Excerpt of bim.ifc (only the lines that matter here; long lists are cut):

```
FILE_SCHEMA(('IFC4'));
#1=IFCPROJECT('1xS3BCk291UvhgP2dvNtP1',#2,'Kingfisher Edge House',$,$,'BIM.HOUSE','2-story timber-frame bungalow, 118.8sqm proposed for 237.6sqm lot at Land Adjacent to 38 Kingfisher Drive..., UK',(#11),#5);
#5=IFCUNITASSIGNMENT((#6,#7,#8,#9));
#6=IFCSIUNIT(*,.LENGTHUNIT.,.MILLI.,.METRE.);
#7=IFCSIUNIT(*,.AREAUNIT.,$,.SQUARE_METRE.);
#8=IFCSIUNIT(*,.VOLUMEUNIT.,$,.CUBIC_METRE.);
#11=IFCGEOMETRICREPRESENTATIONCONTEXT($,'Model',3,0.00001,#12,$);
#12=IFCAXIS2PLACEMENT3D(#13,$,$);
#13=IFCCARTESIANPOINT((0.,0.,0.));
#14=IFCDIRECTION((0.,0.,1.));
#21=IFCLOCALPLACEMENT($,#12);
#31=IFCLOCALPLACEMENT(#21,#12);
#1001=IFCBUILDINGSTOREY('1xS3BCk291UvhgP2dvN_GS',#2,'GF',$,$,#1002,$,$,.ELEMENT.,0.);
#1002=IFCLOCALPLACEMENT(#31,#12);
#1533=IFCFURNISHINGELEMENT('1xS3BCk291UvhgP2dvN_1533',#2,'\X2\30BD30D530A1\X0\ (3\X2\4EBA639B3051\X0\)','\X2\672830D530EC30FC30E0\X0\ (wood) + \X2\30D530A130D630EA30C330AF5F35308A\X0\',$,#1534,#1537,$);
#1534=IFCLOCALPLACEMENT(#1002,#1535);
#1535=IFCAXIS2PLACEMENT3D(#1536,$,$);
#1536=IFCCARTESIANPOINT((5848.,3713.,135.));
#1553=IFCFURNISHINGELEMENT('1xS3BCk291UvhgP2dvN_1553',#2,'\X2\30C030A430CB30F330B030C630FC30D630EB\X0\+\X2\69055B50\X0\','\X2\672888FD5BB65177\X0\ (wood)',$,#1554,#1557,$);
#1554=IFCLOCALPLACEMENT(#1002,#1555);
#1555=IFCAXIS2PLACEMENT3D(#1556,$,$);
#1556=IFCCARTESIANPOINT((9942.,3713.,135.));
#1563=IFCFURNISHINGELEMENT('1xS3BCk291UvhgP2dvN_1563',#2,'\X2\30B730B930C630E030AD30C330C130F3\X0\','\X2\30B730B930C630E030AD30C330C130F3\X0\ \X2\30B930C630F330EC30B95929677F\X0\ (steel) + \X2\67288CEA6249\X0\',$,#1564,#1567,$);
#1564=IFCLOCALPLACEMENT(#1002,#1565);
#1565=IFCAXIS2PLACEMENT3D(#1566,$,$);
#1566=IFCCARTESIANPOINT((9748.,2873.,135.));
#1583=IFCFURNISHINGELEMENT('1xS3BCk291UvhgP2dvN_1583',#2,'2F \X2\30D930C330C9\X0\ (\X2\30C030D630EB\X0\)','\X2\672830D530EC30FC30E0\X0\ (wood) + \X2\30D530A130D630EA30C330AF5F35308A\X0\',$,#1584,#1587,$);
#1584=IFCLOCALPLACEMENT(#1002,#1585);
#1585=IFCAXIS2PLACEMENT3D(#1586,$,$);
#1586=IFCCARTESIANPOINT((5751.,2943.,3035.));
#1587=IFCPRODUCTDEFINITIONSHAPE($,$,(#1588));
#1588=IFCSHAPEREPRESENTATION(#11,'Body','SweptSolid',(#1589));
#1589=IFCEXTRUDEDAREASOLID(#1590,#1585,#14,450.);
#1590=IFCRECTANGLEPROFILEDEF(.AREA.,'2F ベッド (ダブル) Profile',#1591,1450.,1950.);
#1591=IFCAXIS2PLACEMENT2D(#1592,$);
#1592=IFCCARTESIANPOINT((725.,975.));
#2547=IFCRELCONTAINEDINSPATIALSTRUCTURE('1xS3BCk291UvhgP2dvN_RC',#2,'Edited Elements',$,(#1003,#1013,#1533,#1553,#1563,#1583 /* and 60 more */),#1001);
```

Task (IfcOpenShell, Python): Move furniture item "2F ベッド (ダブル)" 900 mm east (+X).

```python
import ifcopenshell
import ifcopenshell.api.geometry
import ifcopenshell.util.placement
import ifcopenshell.util.unit

model = ifcopenshell.open("bim.ifc")
unit_scale = ifcopenshell.util.unit.calculate_unit_scale(model)

item = model.by_guid("1xS3BCk291UvhgP2dvN_1583")
matrix = ifcopenshell.util.placement.get_local_placement(item.ObjectPlacement)
matrix[0, 3] += 0.9 / unit_scale
ifcopenshell.api.geometry.edit_object_placement(model, product=item, matrix=matrix, is_si=False)

print(ifcopenshell.util.placement.get_local_placement(item.ObjectPlacement).round(3) + 0.0)

model.write("bim_v2.ifc")
```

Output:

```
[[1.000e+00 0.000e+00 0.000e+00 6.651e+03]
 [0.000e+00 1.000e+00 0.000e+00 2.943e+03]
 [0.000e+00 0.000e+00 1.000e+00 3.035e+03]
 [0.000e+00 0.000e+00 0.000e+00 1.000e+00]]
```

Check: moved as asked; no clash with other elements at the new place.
